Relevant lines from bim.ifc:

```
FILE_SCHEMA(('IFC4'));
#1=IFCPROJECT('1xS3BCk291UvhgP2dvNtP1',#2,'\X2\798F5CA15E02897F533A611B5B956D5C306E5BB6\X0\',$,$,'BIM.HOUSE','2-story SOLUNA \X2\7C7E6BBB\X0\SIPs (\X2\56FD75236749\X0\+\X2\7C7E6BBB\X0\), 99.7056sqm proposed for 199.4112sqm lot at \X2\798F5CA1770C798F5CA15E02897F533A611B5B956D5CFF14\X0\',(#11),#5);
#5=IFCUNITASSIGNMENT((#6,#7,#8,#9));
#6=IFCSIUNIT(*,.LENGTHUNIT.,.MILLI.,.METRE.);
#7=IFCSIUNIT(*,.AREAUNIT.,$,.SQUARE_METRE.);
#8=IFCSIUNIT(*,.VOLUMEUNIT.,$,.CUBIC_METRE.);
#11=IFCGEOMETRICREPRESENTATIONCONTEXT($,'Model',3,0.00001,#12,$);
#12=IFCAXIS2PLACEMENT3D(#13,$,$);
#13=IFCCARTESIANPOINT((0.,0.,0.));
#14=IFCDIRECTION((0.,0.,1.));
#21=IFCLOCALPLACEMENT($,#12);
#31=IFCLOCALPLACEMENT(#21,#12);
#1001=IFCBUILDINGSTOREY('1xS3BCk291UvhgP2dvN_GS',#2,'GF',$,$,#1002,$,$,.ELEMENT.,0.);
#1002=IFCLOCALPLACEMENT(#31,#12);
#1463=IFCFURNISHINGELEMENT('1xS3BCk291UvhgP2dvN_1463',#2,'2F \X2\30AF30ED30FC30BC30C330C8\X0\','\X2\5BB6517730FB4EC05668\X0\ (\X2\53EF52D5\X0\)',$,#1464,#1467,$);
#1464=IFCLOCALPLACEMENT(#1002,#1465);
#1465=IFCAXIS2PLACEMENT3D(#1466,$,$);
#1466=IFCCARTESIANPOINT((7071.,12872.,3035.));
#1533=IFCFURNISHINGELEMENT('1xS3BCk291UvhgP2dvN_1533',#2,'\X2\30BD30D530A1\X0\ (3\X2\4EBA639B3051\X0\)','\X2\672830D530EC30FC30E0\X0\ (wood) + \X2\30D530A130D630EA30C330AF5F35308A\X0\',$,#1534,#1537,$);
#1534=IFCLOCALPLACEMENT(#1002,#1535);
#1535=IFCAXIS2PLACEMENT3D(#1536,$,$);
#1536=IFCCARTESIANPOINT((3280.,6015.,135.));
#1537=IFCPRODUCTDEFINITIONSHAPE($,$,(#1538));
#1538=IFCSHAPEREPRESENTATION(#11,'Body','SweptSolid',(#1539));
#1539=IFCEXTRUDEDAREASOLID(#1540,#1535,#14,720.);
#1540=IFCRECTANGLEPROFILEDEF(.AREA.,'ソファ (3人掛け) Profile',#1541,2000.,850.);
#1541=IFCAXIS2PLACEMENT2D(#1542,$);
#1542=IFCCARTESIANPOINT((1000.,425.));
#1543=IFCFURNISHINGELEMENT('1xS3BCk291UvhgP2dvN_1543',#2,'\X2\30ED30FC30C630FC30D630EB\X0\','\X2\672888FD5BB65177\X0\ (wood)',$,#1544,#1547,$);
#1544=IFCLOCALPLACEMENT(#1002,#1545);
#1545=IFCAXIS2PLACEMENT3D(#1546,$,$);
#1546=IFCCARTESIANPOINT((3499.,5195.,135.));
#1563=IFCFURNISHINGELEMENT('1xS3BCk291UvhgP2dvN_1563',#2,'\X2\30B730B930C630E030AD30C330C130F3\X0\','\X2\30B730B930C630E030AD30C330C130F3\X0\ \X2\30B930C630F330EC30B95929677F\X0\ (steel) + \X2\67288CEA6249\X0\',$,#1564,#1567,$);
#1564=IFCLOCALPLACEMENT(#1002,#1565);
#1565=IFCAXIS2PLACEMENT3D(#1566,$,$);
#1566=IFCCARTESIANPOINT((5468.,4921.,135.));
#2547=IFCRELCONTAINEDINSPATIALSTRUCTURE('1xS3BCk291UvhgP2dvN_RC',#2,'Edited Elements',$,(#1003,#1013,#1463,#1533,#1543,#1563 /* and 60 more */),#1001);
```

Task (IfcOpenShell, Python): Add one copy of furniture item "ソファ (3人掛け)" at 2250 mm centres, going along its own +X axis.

```python
import ifcopenshell
import ifcopenshell.api.geometry
import ifcopenshell.api.root
import ifcopenshell.util.element
import ifcopenshell.util.placement
import ifcopenshell.util.unit

model = ifcopenshell.open("bim.ifc")
unit_scale = ifcopenshell.util.unit.calculate_unit_scale(model)


def reuse_history(source, copy):
    """copy_class also copies each property set's owner history, people and application; keep the originals."""
    for rel in copy.IsDefinedBy:
        if rel.is_a("IfcRelDefinesByProperties") and (history := rel.RelatingPropertyDefinition.OwnerHistory):
            rel.RelatingPropertyDefinition.OwnerHistory = source.OwnerHistory
            ifcopenshell.util.element.remove_deep2(model, history)


source = model.by_id(1533)
base = ifcopenshell.util.placement.get_local_placement(source.ObjectPlacement)
step = base[:3, 0] * 2.25 / unit_scale

for i in range(1, 2):
    copy = ifcopenshell.api.root.copy_class(model, product=source)
    copy.Representation = ifcopenshell.util.element.copy_deep(
        model, source.Representation, exclude=["IfcGeometricRepresentationContext", "IfcRepresentationMap"]
    )
    reuse_history(source, copy)
    matrix = base.copy()
    matrix[:3, 3] += i * step
    print("added at", matrix[:3, 3].round(3) + 0.0)
    ifcopenshell.api.geometry.edit_object_placement(model, product=copy, matrix=matrix, is_si=False)

model.write("bim_v2.ifc")
```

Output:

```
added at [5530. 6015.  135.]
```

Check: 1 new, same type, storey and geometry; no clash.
